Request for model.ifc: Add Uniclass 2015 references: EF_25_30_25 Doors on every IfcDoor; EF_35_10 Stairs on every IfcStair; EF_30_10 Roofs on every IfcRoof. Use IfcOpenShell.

First a look at what the model holds.

```python
import ifcopenshell

model = ifcopenshell.open("model.ifc")
print(model.schema)
print("classifications:", [c.Name for c in model.by_type("IfcClassification")])
for ifc_class in ("IfcDoor", "IfcRoof", "IfcStair", "IfcWall", "IfcWindow"):
    print(ifc_class, len(model.by_type(ifc_class)))
```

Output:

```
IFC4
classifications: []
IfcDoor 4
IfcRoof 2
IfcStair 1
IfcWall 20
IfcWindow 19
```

```python
import ifcopenshell
import ifcopenshell.api.classification

model = ifcopenshell.open("model.ifc")

system = ifcopenshell.api.classification.add_classification(model, classification="Uniclass 2015")

codes = {
    "IfcDoor": ("EF_25_30_25", "Doors"),
    "IfcStair": ("EF_35_10", "Stairs"),
    "IfcRoof": ("EF_30_10", "Roofs"),
}
for ifc_class, (code, name) in codes.items():
    products = model.by_type(ifc_class)
    ifcopenshell.api.classification.add_reference(
        model, products=products, classification=system, identification=code, name=name
    )
    print(code, len(products))

model.write("model_v2.ifc")
```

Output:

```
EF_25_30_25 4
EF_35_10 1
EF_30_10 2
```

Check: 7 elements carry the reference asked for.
